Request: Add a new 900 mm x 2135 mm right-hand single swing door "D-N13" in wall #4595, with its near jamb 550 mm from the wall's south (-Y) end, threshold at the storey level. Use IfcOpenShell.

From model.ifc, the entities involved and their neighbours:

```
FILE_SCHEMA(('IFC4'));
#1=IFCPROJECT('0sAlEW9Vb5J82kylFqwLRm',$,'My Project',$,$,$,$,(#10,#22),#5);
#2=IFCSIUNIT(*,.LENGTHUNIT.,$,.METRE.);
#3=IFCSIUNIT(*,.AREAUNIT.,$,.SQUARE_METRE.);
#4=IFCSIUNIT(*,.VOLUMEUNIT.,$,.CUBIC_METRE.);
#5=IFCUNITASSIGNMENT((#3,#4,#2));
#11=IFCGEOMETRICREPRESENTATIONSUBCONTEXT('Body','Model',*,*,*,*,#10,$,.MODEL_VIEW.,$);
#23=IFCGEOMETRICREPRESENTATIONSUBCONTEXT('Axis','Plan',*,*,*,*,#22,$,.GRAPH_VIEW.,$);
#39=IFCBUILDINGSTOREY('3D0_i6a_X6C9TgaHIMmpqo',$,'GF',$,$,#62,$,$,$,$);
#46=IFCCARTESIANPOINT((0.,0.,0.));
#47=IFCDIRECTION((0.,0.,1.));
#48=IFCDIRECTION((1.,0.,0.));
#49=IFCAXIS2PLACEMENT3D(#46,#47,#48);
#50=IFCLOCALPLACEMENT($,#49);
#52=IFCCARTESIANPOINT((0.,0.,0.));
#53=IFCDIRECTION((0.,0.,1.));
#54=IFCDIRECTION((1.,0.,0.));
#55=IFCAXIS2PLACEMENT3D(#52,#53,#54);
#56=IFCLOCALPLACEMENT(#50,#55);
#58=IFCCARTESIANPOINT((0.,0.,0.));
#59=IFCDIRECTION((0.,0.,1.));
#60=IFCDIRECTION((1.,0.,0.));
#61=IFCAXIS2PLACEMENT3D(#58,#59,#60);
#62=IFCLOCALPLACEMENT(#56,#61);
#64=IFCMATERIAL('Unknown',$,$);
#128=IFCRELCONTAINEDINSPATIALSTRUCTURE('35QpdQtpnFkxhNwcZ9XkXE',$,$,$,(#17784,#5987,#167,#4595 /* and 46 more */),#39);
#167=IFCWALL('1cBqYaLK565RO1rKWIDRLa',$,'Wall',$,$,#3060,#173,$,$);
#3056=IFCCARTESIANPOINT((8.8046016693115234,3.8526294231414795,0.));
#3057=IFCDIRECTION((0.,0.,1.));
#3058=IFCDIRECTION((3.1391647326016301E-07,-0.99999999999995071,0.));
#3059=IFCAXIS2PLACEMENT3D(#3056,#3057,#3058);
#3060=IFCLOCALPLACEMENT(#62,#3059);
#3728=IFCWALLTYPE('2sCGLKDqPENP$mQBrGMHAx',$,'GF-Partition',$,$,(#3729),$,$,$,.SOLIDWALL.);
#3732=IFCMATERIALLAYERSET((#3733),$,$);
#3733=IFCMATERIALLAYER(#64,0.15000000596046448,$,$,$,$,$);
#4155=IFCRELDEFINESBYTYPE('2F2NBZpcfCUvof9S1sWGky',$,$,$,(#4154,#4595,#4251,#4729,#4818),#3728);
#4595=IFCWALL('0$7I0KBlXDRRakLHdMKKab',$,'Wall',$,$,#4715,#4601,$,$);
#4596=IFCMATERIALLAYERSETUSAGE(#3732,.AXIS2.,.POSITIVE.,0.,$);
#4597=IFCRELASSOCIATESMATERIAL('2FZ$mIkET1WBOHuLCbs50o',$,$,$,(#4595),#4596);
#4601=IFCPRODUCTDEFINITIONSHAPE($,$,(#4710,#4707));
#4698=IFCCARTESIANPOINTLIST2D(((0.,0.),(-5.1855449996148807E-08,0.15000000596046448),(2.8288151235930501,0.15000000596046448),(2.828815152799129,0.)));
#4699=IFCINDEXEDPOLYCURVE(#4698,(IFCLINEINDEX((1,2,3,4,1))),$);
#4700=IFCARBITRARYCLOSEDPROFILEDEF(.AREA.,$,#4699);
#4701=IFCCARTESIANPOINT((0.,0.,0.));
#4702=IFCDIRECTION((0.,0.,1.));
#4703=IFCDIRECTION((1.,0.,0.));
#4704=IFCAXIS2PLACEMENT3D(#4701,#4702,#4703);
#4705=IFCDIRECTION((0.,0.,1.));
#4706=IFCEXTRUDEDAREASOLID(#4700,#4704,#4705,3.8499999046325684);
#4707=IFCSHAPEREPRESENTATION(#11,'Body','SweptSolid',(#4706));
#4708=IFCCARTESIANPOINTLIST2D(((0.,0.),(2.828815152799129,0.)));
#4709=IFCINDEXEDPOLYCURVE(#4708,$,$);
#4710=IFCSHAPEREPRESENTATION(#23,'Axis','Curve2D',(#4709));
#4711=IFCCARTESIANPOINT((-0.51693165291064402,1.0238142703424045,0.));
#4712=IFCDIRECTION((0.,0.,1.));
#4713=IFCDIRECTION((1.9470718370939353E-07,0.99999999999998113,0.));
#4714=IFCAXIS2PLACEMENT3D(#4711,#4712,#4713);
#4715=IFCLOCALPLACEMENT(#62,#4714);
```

```python
import numpy as np
import ifcopenshell
import ifcopenshell.api.feature
import ifcopenshell.api.geometry
import ifcopenshell.api.root
import ifcopenshell.api.spatial
import ifcopenshell.geom
import ifcopenshell.util.element
import ifcopenshell.util.placement
import ifcopenshell.util.representation
import ifcopenshell.util.shape
import ifcopenshell.util.unit

model = ifcopenshell.open("model.ifc")
unit_scale = ifcopenshell.util.unit.calculate_unit_scale(model)
settings = ifcopenshell.geom.settings()


def volume(element):
    """Net volume in cubic metres, openings subtracted."""
    shape = ifcopenshell.geom.create_shape(settings, element)
    return ifcopenshell.util.shape.get_volume(shape.geometry)


wall = model.by_id(4595)
storey = ifcopenshell.util.element.get_container(wall, ifc_class="IfcBuildingStorey")
context = ifcopenshell.util.representation.get_context(model, "Model", "Body", "MODEL_VIEW")
before = volume(wall)

width, height, from_end, sill = 0.9, 2.135, 0.55, 0.0  # metres

# The wall runs along its own X axis, and the end named is its -X end.
wall_shape = ifcopenshell.geom.create_shape(settings, wall)
x, y, z = ifcopenshell.util.shape.get_vertices(wall_shape.geometry).T
start = x.min() + from_end
face, thickness = float(y.min()), float(y.max() - y.min())
wall_matrix = ifcopenshell.util.placement.get_local_placement(wall.ObjectPlacement)
level = ifcopenshell.util.placement.get_local_placement(storey.ObjectPlacement)[2, 3]


def in_wall(x, y):
    """Placement at x, y metres in the wall's axes, at sill height."""
    matrix = wall_matrix.copy()
    matrix[:, 3] = wall_matrix @ np.array([x / unit_scale, y / unit_scale, 0.0, 1.0])
    matrix[2, 3] = level + sill / unit_scale
    return matrix


# Opening: a box that overshoots both wall faces by 50 mm.
opening = ifcopenshell.api.root.create_entity(model, ifc_class="IfcOpeningElement", predefined_type="OPENING")
box = ifcopenshell.api.geometry.add_wall_representation(
    model, context=context, length=width, height=height, thickness=thickness + 0.1
)
ifcopenshell.api.geometry.assign_representation(model, product=opening, representation=box)
ifcopenshell.api.geometry.edit_object_placement(model, product=opening, matrix=in_wall(start, face - 0.05), is_si=False)
ifcopenshell.api.feature.add_feature(model, feature=opening, element=wall)

door = ifcopenshell.api.root.create_entity(model, ifc_class="IfcDoor", name="D-N13", predefined_type="DOOR")
door.OverallWidth, door.OverallHeight = width / unit_scale, height / unit_scale
door.OperationType = "SINGLE_SWING_RIGHT"
body = ifcopenshell.api.geometry.add_door_representation(
    model,
    context=context,
    overall_width=door.OverallWidth,
    overall_height=door.OverallHeight,
    operation_type="SINGLE_SWING_RIGHT",
    lining_properties={"LiningDepth": thickness / unit_scale, "ThresholdDepth": thickness / unit_scale},
)
ifcopenshell.api.geometry.assign_representation(model, product=door, representation=body)
ifcopenshell.api.spatial.assign_container(model, products=[door], relating_structure=storey)
ifcopenshell.api.feature.add_filling(model, opening=opening, element=door)

# The lining spans the wall, so the door starts at the wall face.
ifcopenshell.api.geometry.edit_object_placement(model, product=door, matrix=in_wall(start, face), is_si=False)

after = volume(wall)

print(f"wall volume {before:.3f} -> {after:.3f} m3")

model.write("model_rev.ifc")
```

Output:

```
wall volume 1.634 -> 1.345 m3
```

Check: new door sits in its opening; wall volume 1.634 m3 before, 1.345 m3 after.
